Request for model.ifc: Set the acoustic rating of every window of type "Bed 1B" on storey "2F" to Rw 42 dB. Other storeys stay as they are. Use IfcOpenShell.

First a look at what the model holds.

```python
import ifcopenshell
import ifcopenshell.util.element

model = ifcopenshell.open("model.ifc")
print(model.schema)
storey = next(s for s in model.by_type("IfcBuildingStorey") if s.Name == "2F")
windows = [e for e in ifcopenshell.util.element.get_decomposition(storey) if e.is_a("IfcWindow")]
seen = {}
for e in windows:
    element_type = ifcopenshell.util.element.get_type(e)
    key = (element_type.Name if element_type != e and element_type else None, ifcopenshell.util.element.get_pset(e, "Pset_WindowCommon", "AcousticRating"))
    seen[key] = seen.get(key, 0) + 1
for (name, value), count in sorted(seen.items(), key=str):
    print(count, "x", name, "|", value)
```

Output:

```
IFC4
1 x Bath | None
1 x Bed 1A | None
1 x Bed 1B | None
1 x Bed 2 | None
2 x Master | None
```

```python
import ifcopenshell
import ifcopenshell.api.pset
import ifcopenshell.util.element

model = ifcopenshell.open("model.ifc")

storey = next(s for s in model.by_type("IfcBuildingStorey") if s.Name == "2F")
windows = [e for e in ifcopenshell.util.element.get_decomposition(storey) if e.is_a("IfcWindow")]

count = 0
for e in windows:
    element_type = ifcopenshell.util.element.get_type(e)
    if element_type in (None, e) or element_type.Name != "Bed 1B":
        continue
    # add_pset returns the element's existing set when there is one.
    pset = ifcopenshell.api.pset.add_pset(model, product=e, name="Pset_WindowCommon")
    ifcopenshell.api.pset.edit_pset(model, pset=pset, properties={"AcousticRating": "Rw 42 dB"})
    count += 1

print(count, "windows updated")

model.write("model_v2.ifc")
```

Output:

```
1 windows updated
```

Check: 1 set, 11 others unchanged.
